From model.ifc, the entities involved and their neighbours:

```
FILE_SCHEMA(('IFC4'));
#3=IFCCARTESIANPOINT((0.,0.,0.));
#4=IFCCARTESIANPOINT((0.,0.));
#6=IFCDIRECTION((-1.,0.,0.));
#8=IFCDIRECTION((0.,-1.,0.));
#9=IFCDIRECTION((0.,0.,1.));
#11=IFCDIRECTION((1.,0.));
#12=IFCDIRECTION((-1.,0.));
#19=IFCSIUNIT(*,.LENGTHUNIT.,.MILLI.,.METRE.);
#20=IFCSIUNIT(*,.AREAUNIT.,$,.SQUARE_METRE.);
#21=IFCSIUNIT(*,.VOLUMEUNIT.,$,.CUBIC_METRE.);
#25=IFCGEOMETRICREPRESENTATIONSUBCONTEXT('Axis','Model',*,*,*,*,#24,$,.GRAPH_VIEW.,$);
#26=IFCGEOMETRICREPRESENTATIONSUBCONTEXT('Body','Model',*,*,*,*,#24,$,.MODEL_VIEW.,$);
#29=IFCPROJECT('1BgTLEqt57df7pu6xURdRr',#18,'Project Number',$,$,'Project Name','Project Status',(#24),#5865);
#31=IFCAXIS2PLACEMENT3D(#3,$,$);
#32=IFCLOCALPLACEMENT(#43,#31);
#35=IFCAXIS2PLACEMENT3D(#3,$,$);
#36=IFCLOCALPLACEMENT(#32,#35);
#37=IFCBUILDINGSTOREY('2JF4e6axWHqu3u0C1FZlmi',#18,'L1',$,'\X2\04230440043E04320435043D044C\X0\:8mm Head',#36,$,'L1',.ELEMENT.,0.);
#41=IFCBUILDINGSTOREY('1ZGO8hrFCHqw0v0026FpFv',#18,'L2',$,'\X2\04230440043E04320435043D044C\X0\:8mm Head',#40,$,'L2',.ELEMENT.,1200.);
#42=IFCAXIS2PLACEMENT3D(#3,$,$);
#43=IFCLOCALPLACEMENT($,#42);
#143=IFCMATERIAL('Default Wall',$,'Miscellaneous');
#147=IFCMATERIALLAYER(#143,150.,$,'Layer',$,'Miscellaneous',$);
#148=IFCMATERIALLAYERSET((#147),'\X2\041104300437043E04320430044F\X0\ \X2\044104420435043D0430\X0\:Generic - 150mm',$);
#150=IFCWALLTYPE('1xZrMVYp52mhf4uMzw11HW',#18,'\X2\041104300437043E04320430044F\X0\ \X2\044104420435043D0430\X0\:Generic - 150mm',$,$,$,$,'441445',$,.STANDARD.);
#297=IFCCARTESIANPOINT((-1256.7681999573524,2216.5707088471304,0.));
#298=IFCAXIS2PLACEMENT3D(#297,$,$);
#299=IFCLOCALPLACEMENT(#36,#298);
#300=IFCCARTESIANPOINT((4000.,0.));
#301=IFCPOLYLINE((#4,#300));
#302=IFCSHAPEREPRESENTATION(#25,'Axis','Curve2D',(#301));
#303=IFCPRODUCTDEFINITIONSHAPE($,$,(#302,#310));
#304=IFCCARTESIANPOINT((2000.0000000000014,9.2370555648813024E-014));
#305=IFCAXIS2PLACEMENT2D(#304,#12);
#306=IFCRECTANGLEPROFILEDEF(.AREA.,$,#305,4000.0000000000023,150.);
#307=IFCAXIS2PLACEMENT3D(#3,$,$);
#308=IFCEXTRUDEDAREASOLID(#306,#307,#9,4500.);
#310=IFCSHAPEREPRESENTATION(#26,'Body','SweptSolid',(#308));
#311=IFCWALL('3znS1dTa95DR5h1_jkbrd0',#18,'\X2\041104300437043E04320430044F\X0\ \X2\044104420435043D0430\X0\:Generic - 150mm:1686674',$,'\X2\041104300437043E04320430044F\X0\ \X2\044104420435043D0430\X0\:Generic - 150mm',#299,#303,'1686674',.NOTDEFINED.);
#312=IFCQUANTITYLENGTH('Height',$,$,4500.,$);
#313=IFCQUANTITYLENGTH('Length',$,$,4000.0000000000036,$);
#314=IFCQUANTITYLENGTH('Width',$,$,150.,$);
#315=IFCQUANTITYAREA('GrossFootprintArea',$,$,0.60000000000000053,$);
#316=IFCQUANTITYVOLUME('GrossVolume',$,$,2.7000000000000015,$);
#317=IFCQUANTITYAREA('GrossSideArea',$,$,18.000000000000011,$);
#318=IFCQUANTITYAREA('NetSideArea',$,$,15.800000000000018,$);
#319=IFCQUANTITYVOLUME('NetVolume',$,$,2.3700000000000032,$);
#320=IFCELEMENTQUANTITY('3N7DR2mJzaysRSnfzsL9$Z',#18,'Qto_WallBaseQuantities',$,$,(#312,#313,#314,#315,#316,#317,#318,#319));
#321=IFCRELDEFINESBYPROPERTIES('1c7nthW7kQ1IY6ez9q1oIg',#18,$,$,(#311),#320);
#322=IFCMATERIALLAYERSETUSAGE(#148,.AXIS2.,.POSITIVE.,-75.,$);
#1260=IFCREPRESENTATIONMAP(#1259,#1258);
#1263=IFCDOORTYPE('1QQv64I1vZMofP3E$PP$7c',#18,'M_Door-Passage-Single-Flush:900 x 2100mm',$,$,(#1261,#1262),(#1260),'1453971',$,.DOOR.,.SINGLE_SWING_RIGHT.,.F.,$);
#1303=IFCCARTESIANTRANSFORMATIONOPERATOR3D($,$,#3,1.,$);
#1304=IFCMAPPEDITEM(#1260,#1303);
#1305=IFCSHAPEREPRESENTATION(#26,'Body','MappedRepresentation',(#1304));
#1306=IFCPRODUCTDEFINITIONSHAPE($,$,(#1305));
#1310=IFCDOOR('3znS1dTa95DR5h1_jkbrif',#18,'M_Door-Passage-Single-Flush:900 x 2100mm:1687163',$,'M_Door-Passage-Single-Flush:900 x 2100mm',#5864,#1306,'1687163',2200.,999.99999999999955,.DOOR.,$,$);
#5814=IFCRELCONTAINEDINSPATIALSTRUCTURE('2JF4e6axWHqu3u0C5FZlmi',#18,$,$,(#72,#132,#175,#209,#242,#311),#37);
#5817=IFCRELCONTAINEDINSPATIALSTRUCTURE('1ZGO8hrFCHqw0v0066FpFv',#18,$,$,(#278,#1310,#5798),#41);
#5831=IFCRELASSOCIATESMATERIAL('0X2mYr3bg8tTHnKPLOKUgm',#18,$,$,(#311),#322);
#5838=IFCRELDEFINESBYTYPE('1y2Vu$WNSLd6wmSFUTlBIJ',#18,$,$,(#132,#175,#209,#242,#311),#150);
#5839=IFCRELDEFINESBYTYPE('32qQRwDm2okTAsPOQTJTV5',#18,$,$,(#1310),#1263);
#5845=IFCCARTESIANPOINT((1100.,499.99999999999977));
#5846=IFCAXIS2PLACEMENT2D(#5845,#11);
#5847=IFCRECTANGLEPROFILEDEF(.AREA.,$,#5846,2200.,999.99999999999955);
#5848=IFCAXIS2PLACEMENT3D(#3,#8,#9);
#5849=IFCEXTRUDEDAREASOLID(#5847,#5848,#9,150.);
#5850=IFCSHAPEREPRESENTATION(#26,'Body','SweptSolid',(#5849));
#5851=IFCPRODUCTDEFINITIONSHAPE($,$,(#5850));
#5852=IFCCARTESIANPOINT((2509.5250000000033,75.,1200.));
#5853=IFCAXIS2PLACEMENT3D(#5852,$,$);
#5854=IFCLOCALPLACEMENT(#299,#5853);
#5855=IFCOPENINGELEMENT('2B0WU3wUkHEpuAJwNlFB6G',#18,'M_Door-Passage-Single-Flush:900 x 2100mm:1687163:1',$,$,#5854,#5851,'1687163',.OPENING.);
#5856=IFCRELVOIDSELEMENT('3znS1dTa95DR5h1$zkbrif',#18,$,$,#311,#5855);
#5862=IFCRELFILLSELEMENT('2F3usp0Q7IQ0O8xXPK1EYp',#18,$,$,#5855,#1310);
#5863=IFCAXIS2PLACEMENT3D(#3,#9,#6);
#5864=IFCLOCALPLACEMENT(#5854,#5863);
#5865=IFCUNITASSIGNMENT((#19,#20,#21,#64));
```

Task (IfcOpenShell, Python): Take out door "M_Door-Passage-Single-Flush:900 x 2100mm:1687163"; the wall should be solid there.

```python
import ifcopenshell
import ifcopenshell.api.feature
import ifcopenshell.api.pset
import ifcopenshell.api.root
import ifcopenshell.geom
import ifcopenshell.util.element
import ifcopenshell.util.shape
import ifcopenshell.util.unit

model = ifcopenshell.open("model.ifc")
area_scale = ifcopenshell.util.unit.calculate_unit_scale(model, "AREAUNIT")
volume_scale = ifcopenshell.util.unit.calculate_unit_scale(model, "VOLUMEUNIT")
settings = ifcopenshell.geom.settings()


def volume(element):
    """Net volume in cubic metres, openings subtracted."""
    shape = ifcopenshell.geom.create_shape(settings, element)
    return ifcopenshell.util.shape.get_volume(shape.geometry)


door = model.by_id(1310)
opening = door.FillsVoids[0].RelatingOpeningElement
wall = opening.VoidsElements[0].RelatingBuildingElement
before = volume(wall)

ifcopenshell.api.root.remove_product(model, product=door)
ifcopenshell.api.feature.remove_feature(model, feature=opening)

after = volume(wall)
thickness = 0.15  # wall thickness in metres

# Update the wall's stored quantities.
qto = model.by_id(ifcopenshell.util.element.get_pset(wall, "Qto_WallBaseQuantities", should_inherit=False)["id"])
ifcopenshell.api.pset.edit_qto(model, qto=qto, properties={
    "NetSideArea": after / thickness / area_scale,
    "NetVolume": after / volume_scale,
})

print(f"wall volume {before:.3f} -> {after:.3f} m3")

model.write("model_edited.ifc")
```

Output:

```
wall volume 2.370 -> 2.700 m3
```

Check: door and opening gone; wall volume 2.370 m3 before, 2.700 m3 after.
